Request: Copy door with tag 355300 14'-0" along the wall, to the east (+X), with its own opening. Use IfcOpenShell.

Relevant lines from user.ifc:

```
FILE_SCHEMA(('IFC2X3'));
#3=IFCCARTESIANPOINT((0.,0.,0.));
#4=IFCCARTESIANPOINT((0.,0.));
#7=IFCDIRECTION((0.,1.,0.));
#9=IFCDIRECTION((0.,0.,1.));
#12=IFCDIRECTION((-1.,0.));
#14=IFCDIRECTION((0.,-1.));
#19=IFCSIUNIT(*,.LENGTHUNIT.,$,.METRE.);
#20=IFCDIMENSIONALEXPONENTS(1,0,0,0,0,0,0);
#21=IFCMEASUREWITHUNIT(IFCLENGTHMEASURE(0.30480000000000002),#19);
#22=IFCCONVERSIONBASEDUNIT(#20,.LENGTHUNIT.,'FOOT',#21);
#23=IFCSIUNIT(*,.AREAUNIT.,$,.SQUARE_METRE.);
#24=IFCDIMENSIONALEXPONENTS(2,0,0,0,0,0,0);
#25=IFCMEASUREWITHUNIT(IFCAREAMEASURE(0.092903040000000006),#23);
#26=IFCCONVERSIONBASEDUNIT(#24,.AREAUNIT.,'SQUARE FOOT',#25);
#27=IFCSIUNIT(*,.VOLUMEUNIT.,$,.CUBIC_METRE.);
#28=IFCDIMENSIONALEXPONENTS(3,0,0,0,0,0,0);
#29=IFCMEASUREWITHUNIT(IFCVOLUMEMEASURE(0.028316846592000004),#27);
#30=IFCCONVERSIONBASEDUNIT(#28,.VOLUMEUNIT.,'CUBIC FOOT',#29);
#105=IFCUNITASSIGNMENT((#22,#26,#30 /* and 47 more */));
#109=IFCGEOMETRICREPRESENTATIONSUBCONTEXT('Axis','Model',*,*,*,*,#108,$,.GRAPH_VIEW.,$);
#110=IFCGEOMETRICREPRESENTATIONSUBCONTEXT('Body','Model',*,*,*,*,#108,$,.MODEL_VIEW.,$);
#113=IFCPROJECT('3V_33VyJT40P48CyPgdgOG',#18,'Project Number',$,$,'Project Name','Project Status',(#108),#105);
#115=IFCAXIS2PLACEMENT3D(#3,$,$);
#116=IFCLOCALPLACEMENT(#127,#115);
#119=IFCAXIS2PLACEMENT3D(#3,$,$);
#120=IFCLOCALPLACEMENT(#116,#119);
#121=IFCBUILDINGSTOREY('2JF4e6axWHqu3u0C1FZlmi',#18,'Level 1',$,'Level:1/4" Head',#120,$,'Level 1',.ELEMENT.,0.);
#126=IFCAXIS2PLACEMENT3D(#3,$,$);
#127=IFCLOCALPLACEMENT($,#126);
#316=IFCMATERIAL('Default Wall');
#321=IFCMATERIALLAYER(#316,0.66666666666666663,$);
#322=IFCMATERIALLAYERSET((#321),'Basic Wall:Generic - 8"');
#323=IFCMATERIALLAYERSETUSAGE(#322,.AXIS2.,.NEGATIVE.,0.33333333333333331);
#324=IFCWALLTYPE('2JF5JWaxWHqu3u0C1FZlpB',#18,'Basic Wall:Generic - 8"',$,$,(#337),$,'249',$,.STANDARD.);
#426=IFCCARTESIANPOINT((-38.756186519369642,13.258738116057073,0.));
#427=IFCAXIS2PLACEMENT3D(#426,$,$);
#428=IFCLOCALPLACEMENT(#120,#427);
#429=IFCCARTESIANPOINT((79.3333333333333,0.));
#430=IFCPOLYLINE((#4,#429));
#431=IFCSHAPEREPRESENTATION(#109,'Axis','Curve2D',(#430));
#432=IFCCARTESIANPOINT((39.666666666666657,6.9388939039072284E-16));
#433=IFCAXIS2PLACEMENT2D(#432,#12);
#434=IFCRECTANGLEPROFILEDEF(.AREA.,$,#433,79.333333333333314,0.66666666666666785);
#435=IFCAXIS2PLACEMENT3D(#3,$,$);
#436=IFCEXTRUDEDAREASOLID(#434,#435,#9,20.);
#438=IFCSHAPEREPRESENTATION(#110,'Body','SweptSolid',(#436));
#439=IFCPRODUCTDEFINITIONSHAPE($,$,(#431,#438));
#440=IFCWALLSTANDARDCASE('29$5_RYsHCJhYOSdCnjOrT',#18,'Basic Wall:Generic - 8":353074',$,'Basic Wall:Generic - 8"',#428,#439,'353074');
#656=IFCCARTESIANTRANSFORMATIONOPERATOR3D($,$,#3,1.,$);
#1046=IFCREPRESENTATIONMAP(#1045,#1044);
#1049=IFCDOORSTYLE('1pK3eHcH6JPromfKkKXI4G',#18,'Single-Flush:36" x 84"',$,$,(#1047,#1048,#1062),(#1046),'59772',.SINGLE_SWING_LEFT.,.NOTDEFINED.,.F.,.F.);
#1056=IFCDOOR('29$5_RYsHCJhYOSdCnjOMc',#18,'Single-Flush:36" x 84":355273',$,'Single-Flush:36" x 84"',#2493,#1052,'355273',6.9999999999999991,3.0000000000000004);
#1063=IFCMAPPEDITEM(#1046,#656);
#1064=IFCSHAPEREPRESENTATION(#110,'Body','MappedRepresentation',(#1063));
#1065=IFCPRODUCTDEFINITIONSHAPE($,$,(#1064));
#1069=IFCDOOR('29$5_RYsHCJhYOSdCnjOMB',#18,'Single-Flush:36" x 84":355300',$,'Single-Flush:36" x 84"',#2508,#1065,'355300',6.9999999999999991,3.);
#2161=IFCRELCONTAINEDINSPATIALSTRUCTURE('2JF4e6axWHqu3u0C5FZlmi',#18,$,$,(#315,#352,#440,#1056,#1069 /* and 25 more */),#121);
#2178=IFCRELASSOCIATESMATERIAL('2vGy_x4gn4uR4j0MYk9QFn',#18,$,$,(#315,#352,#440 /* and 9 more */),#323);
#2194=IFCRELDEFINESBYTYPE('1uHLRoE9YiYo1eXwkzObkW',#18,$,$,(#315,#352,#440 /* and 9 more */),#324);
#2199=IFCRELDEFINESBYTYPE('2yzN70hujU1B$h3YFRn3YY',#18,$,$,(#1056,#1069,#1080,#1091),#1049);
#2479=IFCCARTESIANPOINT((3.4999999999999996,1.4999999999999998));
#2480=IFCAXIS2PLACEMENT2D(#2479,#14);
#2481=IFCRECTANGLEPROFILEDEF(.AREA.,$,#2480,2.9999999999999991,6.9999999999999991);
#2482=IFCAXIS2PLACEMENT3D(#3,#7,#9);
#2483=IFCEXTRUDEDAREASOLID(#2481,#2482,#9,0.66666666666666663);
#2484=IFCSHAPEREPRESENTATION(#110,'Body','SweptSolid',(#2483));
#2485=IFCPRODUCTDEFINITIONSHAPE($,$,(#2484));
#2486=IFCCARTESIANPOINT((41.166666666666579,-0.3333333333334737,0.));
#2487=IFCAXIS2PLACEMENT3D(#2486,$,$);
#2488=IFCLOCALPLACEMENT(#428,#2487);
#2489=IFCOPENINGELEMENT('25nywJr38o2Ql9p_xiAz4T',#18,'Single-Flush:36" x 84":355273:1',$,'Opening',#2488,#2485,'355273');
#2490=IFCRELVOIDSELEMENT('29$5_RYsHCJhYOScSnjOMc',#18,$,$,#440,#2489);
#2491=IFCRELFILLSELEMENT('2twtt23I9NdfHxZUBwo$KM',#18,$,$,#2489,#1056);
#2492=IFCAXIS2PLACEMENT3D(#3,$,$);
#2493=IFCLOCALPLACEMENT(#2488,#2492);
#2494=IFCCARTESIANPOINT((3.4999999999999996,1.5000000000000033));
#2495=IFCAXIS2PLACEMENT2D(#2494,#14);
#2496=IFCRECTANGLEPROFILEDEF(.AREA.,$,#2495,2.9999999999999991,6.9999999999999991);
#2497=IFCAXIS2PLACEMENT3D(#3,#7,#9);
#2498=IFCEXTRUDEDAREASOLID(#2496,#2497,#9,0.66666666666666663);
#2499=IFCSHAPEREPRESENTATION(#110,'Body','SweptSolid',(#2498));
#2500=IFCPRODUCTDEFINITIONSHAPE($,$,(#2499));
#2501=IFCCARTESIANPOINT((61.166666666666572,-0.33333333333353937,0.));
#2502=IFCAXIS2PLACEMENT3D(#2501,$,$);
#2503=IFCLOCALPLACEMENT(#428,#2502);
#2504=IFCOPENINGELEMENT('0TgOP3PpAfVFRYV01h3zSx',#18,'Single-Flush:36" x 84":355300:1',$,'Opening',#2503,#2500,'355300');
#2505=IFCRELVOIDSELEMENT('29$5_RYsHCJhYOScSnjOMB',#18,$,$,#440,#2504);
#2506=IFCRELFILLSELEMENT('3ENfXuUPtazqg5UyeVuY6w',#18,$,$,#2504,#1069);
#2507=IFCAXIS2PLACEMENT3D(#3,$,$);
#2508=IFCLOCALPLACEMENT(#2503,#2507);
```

```python
import ifcopenshell
import ifcopenshell.api.feature
import ifcopenshell.api.geometry
import ifcopenshell.api.root
import ifcopenshell.geom
import ifcopenshell.util.element
import ifcopenshell.util.placement
import ifcopenshell.util.shape
import ifcopenshell.util.unit

model = ifcopenshell.open("user.ifc")
unit_scale = ifcopenshell.util.unit.calculate_unit_scale(model)
settings = ifcopenshell.geom.settings()


def volume(element):
    """Net volume in cubic metres, openings subtracted."""
    shape = ifcopenshell.geom.create_shape(settings, element)
    return ifcopenshell.util.shape.get_volume(shape.geometry)


def reuse_history(source, copy):
    """copy_class also copies each property set's owner history, people and application; keep the originals."""
    for rel in copy.IsDefinedBy:
        if rel.is_a("IfcRelDefinesByProperties") and (history := rel.RelatingPropertyDefinition.OwnerHistory):
            rel.RelatingPropertyDefinition.OwnerHistory = source.OwnerHistory
            ifcopenshell.util.element.remove_deep2(model, history)


door = model.by_guid("29$5_RYsHCJhYOSdCnjOMB")
opening = door.FillsVoids[0].RelatingOpeningElement
wall = opening.VoidsElements[0].RelatingBuildingElement
before = volume(wall)
shift = ifcopenshell.util.placement.get_local_placement(wall.ObjectPlacement)[:3, 0] * 168 * 0.0254 / unit_scale

# copy_class copies the void relationship, type, container and properties, but no geometry.
new_opening = ifcopenshell.api.root.copy_class(model, product=opening)
new_opening.Representation = ifcopenshell.util.element.copy_deep(
    model, opening.Representation, exclude=["IfcGeometricRepresentationContext", "IfcRepresentationMap"]
)
new_opening.Name = 'Single-Flush:36" x 84"'
new_opening.Tag = None
new_door = ifcopenshell.api.root.copy_class(model, product=door)
new_door.Representation = ifcopenshell.util.element.copy_deep(
    model, door.Representation, exclude=["IfcGeometricRepresentationContext", "IfcRepresentationMap"]
)
new_door.Name = 'Single-Flush:36" x 84"'
new_door.Tag = None
reuse_history(door, new_door)
fills = ifcopenshell.api.feature.add_filling(model, opening=new_opening, element=new_door)
fills.OwnerHistory = new_door.OwnerHistory  # required in IFC2X3

for old, new in ((opening, new_opening), (door, new_door)):
    matrix = ifcopenshell.util.placement.get_local_placement(old.ObjectPlacement)
    matrix[:3, 3] += shift
    ifcopenshell.api.geometry.edit_object_placement(model, product=new, matrix=matrix, is_si=False)

after = volume(wall)

print(f"wall volume {before:.3f} -> {after:.3f} m3")

model.write("user-out.ifc")
```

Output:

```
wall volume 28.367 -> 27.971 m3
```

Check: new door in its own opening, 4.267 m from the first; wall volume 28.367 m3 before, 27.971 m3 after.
